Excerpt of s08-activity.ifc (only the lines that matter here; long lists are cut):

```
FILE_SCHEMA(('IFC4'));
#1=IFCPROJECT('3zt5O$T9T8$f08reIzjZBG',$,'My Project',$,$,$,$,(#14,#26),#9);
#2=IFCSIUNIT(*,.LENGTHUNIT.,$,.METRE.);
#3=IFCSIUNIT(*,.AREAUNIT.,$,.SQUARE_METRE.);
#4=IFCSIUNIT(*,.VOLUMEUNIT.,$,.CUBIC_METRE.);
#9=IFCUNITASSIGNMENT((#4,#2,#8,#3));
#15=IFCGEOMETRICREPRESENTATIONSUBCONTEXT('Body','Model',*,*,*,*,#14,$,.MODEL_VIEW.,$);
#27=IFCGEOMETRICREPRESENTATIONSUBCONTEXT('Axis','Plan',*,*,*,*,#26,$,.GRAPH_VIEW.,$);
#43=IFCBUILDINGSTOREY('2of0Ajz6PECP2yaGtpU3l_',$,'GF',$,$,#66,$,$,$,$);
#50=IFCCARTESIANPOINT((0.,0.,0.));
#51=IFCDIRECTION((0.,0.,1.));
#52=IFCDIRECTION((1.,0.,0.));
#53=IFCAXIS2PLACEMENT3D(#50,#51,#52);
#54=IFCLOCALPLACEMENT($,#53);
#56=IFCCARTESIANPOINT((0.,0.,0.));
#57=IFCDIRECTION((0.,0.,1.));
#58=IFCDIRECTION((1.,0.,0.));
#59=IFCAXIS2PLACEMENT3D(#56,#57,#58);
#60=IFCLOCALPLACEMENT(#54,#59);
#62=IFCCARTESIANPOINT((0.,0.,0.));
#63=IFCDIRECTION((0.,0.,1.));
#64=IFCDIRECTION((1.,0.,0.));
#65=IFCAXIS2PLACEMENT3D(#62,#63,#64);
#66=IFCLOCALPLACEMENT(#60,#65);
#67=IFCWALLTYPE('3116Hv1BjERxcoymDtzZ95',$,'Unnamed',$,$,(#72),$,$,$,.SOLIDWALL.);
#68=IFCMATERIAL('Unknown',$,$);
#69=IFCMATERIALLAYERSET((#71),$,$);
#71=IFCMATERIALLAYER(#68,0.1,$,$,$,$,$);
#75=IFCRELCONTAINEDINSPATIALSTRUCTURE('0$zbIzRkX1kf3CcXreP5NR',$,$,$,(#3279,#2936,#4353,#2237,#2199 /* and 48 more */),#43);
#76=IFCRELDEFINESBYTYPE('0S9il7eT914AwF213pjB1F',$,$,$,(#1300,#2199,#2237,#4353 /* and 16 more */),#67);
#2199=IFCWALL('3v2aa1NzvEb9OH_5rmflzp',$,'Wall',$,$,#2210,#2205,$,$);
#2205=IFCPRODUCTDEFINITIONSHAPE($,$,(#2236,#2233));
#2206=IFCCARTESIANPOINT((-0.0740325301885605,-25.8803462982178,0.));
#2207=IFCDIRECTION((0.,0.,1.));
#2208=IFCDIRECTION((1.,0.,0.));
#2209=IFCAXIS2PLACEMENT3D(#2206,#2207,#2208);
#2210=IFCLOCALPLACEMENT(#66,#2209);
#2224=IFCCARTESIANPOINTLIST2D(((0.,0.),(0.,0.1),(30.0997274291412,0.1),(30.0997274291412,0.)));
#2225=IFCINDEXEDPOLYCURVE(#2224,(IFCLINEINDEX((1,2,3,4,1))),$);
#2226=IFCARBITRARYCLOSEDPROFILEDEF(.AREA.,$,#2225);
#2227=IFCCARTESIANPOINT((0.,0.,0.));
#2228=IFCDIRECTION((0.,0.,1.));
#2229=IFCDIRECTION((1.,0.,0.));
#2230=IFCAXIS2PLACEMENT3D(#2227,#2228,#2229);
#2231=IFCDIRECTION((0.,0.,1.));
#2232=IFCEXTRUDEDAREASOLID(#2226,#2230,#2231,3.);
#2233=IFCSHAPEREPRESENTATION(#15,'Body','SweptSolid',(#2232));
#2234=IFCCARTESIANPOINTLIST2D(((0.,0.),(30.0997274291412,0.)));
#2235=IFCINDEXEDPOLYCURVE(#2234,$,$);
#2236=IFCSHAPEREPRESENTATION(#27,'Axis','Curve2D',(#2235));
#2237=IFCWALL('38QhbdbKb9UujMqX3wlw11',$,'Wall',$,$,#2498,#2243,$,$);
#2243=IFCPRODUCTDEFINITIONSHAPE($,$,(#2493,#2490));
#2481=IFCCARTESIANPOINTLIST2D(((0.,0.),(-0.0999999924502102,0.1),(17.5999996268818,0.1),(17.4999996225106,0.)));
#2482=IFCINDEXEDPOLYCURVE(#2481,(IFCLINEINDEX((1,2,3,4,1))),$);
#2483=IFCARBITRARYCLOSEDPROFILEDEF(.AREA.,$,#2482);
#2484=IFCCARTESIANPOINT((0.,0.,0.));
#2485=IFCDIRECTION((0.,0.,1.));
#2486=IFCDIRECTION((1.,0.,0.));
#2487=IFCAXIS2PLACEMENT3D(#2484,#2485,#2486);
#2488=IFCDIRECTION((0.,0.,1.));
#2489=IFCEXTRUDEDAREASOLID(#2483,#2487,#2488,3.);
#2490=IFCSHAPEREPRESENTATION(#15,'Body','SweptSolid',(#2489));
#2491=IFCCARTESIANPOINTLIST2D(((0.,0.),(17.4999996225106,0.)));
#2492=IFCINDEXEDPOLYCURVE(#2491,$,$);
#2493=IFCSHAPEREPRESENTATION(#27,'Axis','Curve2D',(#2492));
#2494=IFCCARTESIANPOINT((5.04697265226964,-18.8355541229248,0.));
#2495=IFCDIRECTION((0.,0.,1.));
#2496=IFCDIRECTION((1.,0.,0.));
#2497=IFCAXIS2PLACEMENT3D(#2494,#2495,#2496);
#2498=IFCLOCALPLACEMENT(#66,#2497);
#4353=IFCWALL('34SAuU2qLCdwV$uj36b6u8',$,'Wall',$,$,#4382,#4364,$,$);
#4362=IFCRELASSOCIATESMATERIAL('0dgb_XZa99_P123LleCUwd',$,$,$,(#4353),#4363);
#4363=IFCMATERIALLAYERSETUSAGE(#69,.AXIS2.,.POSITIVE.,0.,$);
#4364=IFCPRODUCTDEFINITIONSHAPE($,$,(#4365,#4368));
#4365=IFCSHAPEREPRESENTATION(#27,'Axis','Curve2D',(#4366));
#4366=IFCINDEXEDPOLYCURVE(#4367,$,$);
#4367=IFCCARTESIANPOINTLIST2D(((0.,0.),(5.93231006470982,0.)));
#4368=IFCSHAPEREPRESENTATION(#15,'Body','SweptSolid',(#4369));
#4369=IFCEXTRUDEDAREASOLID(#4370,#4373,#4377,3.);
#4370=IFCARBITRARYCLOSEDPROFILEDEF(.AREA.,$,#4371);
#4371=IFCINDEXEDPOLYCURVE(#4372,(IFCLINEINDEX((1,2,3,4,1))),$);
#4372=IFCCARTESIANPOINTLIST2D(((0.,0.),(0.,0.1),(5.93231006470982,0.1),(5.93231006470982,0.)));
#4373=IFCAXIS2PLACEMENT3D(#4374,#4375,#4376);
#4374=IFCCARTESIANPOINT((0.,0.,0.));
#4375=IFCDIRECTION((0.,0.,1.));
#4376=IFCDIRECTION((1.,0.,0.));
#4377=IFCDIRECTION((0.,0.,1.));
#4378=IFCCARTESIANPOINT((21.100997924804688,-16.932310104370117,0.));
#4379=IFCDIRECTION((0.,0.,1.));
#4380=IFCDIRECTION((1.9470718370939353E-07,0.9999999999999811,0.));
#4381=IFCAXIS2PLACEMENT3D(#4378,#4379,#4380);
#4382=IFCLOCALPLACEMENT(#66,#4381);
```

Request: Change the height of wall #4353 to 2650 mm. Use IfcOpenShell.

```python
import ifcopenshell
import ifcopenshell.geom
import ifcopenshell.util.representation
import ifcopenshell.util.shape
import ifcopenshell.util.unit

model = ifcopenshell.open("s08-activity.ifc")
unit_scale = ifcopenshell.util.unit.calculate_unit_scale(model)
settings = ifcopenshell.geom.settings()


def volume(element):
    """Net volume in cubic metres, openings subtracted."""
    shape = ifcopenshell.geom.create_shape(settings, element)
    return ifcopenshell.util.shape.get_volume(shape.geometry)


wall = model.by_id(4353)
before = volume(wall)

body = ifcopenshell.util.representation.get_representation(wall, "Model", "Body")
solid = body.Items[0]
old_height = solid.Depth
solid.Depth = 2.65 / unit_scale
after = volume(wall)

print(f"height {old_height:g} -> {solid.Depth:g}, volume {before:.3f} -> {after:.3f} m3")

model.write("s08-activity_updated.ifc")
```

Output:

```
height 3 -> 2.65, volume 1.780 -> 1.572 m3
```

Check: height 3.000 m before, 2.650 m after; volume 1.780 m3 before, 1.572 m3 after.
